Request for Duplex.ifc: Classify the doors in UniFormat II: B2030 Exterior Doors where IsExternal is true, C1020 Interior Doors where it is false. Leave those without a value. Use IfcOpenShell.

First a look at what the model holds.

```python
import ifcopenshell
import ifcopenshell.util.element

model = ifcopenshell.open("Duplex.ifc")
print(model.schema)
print("classifications:", [c.Name for c in model.by_type("IfcClassification")])
values = [ifcopenshell.util.element.get_pset(e, "Pset_DoorCommon", "IsExternal") for e in model.by_type("IfcDoor")]
for value in (True, False, None):
    print("IsExternal", value, values.count(value))
```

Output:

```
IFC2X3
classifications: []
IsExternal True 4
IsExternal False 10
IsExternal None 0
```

```python
import ifcopenshell
import ifcopenshell.api.classification
import ifcopenshell.util.element

model = ifcopenshell.open("Duplex.ifc")

# IFC2X3 requires Source and Edition and has no link from the project to the system.
system = model.create_entity("IfcClassification", Source="ASTM", Edition="E1557", Name="UniFormat II")

doors = model.by_type("IfcDoor")
external = {e: ifcopenshell.util.element.get_pset(e, "Pset_DoorCommon", "IsExternal") for e in doors}
for flag, code, name in ((True, "B2030", "Exterior Doors"), (False, "C1020", "Interior Doors")):
    products = [e for e in doors if external[e] is flag]
    ifcopenshell.api.classification.add_reference(
        model, products=products, classification=system, identification=code, name=name
    )
    print(code, len(products))

model.write("Duplex_updated.ifc")
```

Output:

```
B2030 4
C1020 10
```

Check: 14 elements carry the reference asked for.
